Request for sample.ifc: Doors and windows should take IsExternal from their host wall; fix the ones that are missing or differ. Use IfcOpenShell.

First a look at what the model holds.

```python
import ifcopenshell
import ifcopenshell.util.element

model = ifcopenshell.open("sample.ifc")
print(model.schema)
seen = {}
for e in model.by_type("IfcDoor") + model.by_type("IfcWindow"):
    if not e.FillsVoids:
        continue
    host = e.FillsVoids[0].RelatingOpeningElement.VoidsElements[0].RelatingBuildingElement
    own = ifcopenshell.util.element.get_pset(e, f"Pset_{e.is_a()[3:].removesuffix('StandardCase')}Common", "IsExternal")
    wall = ifcopenshell.util.element.get_pset(host, "Pset_WallCommon", "IsExternal")
    seen[e.is_a(), own, wall] = seen.get((e.is_a(), own, wall), 0) + 1
for (cls, own, wall), count in sorted(seen.items(), key=str):
    print(count, cls, "IsExternal:", own, "| host wall:", wall)
```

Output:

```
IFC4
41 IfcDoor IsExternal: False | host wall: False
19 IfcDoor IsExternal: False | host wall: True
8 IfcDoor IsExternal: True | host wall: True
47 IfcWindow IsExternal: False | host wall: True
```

```python
import ifcopenshell
import ifcopenshell.api.pset
import ifcopenshell.util.element

model = ifcopenshell.open("sample.ifc")

count = 0
for ifc_class, pset_name in (("IfcDoor", "Pset_DoorCommon"), ("IfcWindow", "Pset_WindowCommon")):
    for e in model.by_type(ifc_class):
        if not e.FillsVoids:
            continue
        host = e.FillsVoids[0].RelatingOpeningElement.VoidsElements[0].RelatingBuildingElement
        external = ifcopenshell.util.element.get_pset(host, "Pset_WallCommon", "IsExternal")
        if external is None or ifcopenshell.util.element.get_pset(e, pset_name, "IsExternal") == external:
            continue
        pset = ifcopenshell.api.pset.add_pset(model, product=e, name=pset_name)
        ifcopenshell.api.pset.edit_pset(model, pset=pset, properties={"IsExternal": external})
        count += 1

print(count, "updated")

model.write("sample-out.ifc")
```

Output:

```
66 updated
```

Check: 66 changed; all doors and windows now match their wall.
